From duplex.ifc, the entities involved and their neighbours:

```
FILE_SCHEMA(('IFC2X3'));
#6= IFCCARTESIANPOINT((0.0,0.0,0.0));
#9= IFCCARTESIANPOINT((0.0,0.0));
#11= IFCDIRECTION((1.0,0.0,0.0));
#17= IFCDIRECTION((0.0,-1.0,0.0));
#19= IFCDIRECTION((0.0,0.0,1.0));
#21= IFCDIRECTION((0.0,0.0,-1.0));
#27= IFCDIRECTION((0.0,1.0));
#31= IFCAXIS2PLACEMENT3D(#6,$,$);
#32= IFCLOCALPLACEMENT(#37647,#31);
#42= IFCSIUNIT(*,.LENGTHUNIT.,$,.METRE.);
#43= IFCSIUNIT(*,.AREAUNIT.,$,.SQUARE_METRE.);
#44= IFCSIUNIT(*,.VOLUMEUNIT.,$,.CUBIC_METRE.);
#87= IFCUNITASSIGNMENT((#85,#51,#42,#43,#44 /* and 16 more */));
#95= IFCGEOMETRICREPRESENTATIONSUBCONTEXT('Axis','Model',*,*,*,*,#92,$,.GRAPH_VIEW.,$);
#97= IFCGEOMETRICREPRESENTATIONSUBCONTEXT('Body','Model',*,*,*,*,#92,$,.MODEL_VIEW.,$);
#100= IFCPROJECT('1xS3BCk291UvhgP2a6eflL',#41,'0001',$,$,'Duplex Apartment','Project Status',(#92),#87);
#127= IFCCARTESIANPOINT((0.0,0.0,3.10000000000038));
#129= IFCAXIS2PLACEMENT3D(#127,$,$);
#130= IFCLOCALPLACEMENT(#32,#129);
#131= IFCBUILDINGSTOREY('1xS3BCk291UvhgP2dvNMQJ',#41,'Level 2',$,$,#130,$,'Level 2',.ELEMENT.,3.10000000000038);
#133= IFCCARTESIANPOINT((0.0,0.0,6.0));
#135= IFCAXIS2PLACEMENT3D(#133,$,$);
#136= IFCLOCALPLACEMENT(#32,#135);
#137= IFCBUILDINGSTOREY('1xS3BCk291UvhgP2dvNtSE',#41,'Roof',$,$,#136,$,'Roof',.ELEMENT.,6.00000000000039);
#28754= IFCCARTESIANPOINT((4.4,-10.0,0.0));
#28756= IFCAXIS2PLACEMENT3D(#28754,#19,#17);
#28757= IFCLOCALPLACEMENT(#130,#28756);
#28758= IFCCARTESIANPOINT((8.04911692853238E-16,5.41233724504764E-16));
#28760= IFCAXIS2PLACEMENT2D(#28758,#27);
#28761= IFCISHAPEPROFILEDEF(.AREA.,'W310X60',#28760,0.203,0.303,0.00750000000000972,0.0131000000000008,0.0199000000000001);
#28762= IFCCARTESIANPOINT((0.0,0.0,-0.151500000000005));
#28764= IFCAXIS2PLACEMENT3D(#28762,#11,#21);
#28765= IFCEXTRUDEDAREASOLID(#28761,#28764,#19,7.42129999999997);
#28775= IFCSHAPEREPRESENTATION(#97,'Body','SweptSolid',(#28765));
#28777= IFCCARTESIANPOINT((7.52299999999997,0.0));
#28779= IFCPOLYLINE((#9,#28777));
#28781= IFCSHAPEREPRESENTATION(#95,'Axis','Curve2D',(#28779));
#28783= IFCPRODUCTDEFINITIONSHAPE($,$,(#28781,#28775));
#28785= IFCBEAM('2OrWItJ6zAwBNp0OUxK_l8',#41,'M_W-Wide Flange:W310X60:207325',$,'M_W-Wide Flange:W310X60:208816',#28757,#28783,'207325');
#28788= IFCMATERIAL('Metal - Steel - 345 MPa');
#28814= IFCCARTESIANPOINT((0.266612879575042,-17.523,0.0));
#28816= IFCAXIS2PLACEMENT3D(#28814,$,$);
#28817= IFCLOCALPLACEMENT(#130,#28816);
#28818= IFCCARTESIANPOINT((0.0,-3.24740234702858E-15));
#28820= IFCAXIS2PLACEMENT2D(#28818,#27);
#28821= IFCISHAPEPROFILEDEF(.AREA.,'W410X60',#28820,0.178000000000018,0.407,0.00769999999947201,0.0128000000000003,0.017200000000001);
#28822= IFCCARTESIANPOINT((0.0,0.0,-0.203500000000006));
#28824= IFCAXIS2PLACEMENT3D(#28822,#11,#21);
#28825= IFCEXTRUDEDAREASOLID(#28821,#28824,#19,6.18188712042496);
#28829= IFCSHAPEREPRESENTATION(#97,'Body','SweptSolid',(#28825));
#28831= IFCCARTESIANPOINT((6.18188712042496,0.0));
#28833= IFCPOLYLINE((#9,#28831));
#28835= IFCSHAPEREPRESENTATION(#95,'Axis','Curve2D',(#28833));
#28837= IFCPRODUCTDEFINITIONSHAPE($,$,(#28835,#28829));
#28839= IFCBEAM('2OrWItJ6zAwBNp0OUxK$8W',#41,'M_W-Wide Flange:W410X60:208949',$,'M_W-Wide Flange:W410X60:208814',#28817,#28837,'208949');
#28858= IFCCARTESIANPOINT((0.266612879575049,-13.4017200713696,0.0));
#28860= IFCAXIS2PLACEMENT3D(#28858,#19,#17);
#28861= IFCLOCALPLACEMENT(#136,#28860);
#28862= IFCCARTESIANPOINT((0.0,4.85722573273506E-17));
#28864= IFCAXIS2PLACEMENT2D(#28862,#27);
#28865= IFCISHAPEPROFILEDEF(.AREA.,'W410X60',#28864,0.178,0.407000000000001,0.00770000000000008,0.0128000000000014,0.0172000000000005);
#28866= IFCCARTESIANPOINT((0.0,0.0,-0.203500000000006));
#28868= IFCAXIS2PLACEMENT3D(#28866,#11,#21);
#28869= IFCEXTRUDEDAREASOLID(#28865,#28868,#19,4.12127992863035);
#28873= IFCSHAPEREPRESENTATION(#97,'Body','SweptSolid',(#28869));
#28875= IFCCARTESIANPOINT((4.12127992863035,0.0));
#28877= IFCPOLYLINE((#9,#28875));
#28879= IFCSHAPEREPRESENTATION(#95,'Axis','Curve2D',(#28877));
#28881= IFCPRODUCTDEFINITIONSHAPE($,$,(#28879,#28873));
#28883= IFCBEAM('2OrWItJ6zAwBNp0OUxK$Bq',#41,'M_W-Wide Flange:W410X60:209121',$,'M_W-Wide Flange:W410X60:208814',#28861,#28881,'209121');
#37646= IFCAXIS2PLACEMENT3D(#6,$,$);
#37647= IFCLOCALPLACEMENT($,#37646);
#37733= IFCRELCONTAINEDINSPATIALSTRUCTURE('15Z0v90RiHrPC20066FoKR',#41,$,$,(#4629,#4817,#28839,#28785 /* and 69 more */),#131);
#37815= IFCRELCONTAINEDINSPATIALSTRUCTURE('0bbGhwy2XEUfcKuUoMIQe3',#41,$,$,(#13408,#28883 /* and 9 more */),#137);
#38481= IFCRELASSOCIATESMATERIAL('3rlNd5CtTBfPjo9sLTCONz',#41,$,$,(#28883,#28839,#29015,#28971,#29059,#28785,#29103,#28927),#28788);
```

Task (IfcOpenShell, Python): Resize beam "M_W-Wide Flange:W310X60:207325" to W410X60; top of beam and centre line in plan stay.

```python
import ifcopenshell
import ifcopenshell.util.element
import ifcopenshell.util.representation

model = ifcopenshell.open("duplex.ifc")

member = model.by_id(28785)
source = next(p for p in model.by_type("IfcIShapeProfileDef") if p.ProfileName == "W410X60")

body = ifcopenshell.util.representation.get_representation(member, "Model", "Body")
solid = body.Items[0]
old_profile = solid.SweptArea

# Copy the section's sizes but keep this member's own profile position.
profile = ifcopenshell.util.element.copy(model, source)
# Profiles are centred, so shift by half the change in depth to hold the top.
shift = (old_profile.OverallDepth - profile.OverallDepth) / 2
x, y = old_profile.Position.Location.Coordinates
up = (-1.0, 0.0)  # upwards, in the solid's own plane
location = model.createIfcCartesianPoint((x + up[0] * shift, y + up[1] * shift))
profile.Position = model.createIfcAxis2Placement2D(location, old_profile.Position.RefDirection)
solid.SweptArea = profile
if not model.get_total_inverses(old_profile):
    ifcopenshell.util.element.remove_deep2(model, old_profile)
member.Name = member.Name.replace("W310X60", "W410X60")
member.ObjectType = member.ObjectType.replace("W310X60", "W410X60")

print(solid.SweptArea)

model.write("duplex_updated.ifc")
```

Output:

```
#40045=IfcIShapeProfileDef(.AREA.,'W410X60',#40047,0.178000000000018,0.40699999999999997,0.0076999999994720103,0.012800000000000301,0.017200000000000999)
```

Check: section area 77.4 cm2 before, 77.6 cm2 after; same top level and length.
